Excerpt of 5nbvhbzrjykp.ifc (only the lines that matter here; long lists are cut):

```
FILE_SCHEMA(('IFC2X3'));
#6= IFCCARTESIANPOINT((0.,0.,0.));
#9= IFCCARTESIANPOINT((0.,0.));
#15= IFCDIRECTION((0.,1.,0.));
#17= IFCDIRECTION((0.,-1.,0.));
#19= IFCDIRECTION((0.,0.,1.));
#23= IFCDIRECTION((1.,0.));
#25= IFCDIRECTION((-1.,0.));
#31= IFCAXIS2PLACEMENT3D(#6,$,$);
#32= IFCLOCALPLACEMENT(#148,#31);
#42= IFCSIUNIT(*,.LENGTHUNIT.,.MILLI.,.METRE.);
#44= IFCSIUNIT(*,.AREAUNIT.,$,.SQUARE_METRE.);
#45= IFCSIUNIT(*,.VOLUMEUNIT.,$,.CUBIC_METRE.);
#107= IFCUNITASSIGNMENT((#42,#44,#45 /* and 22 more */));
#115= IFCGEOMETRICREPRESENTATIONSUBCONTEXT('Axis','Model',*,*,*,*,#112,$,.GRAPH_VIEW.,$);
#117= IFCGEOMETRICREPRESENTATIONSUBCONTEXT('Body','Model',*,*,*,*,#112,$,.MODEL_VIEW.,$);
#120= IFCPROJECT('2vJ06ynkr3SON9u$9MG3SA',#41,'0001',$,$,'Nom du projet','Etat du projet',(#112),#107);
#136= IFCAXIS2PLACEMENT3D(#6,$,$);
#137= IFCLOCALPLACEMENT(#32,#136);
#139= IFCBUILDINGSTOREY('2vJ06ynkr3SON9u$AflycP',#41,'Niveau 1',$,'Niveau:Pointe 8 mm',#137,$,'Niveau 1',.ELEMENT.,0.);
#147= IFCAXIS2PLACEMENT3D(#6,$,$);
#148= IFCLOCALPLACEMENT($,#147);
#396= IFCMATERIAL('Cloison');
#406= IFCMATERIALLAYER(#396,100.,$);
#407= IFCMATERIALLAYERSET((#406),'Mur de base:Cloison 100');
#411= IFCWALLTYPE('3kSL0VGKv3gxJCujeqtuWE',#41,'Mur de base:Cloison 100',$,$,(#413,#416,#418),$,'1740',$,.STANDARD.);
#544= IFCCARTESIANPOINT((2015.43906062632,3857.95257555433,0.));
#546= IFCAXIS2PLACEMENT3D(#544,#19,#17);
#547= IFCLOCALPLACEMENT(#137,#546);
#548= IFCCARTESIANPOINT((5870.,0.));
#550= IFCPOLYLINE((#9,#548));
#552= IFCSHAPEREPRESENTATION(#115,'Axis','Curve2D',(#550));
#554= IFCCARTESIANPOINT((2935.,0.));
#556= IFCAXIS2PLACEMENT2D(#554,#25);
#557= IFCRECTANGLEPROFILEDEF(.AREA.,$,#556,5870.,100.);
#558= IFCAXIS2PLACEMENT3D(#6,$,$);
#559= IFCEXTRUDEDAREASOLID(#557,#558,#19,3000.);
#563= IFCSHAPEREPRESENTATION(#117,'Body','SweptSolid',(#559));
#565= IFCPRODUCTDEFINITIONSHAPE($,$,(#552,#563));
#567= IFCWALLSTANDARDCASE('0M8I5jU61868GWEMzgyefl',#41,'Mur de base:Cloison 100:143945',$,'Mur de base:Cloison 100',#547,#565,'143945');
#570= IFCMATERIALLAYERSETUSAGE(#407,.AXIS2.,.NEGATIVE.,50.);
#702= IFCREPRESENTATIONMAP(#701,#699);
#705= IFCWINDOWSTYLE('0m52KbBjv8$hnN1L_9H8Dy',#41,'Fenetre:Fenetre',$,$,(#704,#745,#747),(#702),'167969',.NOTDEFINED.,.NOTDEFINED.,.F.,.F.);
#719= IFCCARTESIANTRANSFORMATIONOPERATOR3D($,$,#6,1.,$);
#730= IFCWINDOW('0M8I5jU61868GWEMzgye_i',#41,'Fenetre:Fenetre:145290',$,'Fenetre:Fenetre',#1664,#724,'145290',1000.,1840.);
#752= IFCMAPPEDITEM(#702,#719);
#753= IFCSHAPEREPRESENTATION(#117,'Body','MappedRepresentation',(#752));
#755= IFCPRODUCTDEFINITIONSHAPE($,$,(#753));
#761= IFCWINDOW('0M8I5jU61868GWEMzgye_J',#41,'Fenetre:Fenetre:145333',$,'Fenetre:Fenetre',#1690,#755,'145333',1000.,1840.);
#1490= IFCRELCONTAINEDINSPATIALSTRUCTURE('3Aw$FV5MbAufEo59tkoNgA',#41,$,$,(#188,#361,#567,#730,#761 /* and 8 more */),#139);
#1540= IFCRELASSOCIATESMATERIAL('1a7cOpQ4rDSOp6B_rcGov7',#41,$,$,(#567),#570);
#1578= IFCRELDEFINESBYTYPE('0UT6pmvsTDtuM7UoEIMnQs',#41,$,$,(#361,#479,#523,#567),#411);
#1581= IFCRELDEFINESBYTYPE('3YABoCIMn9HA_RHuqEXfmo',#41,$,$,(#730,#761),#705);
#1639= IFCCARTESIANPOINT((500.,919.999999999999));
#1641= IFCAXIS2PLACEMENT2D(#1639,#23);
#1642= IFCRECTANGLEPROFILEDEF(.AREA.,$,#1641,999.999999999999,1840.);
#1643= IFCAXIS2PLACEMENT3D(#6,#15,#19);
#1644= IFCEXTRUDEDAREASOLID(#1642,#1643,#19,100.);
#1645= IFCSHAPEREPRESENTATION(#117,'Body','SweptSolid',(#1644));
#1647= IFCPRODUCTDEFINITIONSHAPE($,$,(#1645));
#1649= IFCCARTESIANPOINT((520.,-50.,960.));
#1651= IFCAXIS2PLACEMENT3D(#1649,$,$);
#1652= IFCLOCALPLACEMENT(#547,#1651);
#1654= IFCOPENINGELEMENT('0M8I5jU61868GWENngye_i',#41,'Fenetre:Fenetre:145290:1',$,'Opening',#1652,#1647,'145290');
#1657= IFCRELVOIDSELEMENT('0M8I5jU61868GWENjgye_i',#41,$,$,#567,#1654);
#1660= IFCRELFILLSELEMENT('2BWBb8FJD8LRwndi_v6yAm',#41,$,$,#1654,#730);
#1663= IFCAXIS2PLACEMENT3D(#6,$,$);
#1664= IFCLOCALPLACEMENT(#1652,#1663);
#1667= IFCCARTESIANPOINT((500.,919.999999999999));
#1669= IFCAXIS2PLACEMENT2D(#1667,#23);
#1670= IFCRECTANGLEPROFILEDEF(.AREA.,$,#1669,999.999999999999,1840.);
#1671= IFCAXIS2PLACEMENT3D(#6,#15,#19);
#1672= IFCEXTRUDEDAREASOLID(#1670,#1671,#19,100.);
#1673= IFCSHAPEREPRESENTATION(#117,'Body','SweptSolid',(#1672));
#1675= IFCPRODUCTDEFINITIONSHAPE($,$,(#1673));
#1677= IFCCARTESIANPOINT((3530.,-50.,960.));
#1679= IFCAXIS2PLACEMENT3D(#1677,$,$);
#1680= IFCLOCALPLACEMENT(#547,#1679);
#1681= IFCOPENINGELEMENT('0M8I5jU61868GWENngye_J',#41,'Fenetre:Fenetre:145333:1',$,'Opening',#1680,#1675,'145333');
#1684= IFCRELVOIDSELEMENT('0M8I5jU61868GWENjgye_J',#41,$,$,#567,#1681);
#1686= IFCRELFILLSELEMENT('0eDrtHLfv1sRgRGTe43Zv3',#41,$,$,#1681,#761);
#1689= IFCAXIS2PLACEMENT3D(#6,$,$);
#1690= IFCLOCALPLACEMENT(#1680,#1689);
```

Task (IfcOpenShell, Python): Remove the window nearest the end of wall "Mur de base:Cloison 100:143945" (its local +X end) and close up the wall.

```python
import ifcopenshell
import ifcopenshell.api.feature
import ifcopenshell.api.root
import ifcopenshell.geom
import ifcopenshell.util.shape

model = ifcopenshell.open("5nbvhbzrjykp.ifc")
settings = ifcopenshell.geom.settings()


def volume(element):
    """Net volume in cubic metres, openings subtracted."""
    shape = ifcopenshell.geom.create_shape(settings, element)
    return ifcopenshell.util.shape.get_volume(shape.geometry)


window = model.by_id(761)
opening = window.FillsVoids[0].RelatingOpeningElement
wall = opening.VoidsElements[0].RelatingBuildingElement
before = volume(wall)

ifcopenshell.api.root.remove_product(model, product=window)
ifcopenshell.api.feature.remove_feature(model, feature=opening)

after = volume(wall)

print(f"wall volume {before:.3f} -> {after:.3f} m3")

model.write("5nbvhbzrjykp_updated.ifc")
```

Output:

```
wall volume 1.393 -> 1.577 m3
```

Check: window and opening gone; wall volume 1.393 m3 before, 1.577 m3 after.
